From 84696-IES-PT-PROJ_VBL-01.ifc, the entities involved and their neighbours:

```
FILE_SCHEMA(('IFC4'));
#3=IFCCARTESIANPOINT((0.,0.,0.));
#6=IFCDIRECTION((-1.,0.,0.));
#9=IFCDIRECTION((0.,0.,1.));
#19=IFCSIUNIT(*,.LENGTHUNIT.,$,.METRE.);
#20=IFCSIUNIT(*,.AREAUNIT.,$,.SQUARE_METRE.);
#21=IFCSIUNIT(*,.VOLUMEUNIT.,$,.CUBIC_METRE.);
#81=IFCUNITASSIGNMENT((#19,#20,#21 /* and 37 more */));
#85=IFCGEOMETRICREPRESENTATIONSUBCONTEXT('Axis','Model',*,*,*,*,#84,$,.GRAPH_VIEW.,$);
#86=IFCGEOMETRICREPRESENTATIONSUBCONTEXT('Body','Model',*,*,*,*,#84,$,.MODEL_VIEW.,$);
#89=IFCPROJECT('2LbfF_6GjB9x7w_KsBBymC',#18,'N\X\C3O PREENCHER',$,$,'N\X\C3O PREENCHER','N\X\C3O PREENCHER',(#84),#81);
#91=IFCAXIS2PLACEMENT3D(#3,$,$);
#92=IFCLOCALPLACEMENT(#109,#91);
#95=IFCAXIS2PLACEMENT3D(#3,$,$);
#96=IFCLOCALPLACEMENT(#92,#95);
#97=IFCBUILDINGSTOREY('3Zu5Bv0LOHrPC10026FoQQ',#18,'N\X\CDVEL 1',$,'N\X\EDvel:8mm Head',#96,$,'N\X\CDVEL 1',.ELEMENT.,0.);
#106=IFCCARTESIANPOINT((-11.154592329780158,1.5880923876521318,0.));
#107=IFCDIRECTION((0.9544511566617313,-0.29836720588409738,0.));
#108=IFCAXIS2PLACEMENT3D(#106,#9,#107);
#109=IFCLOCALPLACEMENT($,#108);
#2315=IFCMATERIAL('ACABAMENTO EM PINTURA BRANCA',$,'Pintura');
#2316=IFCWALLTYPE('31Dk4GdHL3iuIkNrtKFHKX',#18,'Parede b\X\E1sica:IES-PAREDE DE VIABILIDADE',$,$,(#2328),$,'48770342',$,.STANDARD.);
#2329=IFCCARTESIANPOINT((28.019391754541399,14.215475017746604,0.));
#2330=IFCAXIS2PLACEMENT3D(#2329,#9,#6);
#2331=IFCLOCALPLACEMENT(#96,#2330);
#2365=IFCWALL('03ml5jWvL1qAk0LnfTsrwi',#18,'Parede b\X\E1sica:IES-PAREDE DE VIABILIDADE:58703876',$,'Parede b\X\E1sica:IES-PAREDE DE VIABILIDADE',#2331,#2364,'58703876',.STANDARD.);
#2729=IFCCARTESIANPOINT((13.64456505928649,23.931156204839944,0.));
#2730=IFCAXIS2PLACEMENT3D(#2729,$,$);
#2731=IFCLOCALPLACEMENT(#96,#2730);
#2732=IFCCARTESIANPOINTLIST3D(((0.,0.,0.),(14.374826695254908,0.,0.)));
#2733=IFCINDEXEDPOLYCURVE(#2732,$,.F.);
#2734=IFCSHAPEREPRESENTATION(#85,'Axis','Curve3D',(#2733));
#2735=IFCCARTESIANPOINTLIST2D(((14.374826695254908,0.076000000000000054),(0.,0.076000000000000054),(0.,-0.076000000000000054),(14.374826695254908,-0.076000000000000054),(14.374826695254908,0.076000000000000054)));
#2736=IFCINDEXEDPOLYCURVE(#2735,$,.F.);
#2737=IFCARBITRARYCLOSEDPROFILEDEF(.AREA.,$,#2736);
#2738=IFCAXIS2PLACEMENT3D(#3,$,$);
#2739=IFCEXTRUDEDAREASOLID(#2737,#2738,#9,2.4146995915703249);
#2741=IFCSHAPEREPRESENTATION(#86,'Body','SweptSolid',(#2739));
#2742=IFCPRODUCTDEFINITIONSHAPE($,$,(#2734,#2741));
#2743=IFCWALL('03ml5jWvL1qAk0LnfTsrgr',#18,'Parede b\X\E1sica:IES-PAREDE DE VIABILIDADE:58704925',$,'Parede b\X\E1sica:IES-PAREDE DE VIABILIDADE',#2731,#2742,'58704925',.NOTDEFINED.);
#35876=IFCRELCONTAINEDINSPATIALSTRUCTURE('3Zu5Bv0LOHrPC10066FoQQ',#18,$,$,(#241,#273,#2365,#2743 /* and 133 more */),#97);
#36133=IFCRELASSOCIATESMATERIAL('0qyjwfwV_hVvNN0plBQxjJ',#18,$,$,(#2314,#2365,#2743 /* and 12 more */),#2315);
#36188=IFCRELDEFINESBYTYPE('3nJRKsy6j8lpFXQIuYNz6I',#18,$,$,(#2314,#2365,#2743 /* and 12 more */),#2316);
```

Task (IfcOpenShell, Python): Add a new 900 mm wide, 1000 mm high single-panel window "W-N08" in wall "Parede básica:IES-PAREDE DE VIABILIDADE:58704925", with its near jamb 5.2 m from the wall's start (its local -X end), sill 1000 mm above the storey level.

```python
import numpy as np
import ifcopenshell
import ifcopenshell.api.feature
import ifcopenshell.api.geometry
import ifcopenshell.api.root
import ifcopenshell.api.spatial
import ifcopenshell.geom
import ifcopenshell.util.element
import ifcopenshell.util.placement
import ifcopenshell.util.representation
import ifcopenshell.util.shape
import ifcopenshell.util.unit

model = ifcopenshell.open("84696-IES-PT-PROJ_VBL-01.ifc")
unit_scale = ifcopenshell.util.unit.calculate_unit_scale(model)
settings = ifcopenshell.geom.settings()


def volume(element):
    """Net volume in cubic metres, openings subtracted."""
    shape = ifcopenshell.geom.create_shape(settings, element)
    return ifcopenshell.util.shape.get_volume(shape.geometry)


wall = model.by_id(2743)
storey = ifcopenshell.util.element.get_container(wall, ifc_class="IfcBuildingStorey")
context = ifcopenshell.util.representation.get_context(model, "Model", "Body", "MODEL_VIEW")
before = volume(wall)

width, height, from_end, sill = 0.9, 1, 5.2, 1  # metres

# The wall runs along its own X axis, and the end named is its -X end.
wall_shape = ifcopenshell.geom.create_shape(settings, wall)
x, y, z = ifcopenshell.util.shape.get_vertices(wall_shape.geometry).T
start = x.min() + from_end
face, thickness = float(y.min()), float(y.max() - y.min())
wall_matrix = ifcopenshell.util.placement.get_local_placement(wall.ObjectPlacement)
level = ifcopenshell.util.placement.get_local_placement(storey.ObjectPlacement)[2, 3]


def in_wall(x, y):
    """Placement at x, y metres in the wall's axes, at sill height."""
    matrix = wall_matrix.copy()
    matrix[:, 3] = wall_matrix @ np.array([x / unit_scale, y / unit_scale, 0.0, 1.0])
    matrix[2, 3] = level + sill / unit_scale
    return matrix


# Opening: a box that overshoots both wall faces by 50 mm.
opening = ifcopenshell.api.root.create_entity(model, ifc_class="IfcOpeningElement", predefined_type="OPENING")
box = ifcopenshell.api.geometry.add_wall_representation(
    model, context=context, length=width, height=height, thickness=thickness + 0.1
)
ifcopenshell.api.geometry.assign_representation(model, product=opening, representation=box)
ifcopenshell.api.geometry.edit_object_placement(model, product=opening, matrix=in_wall(start, face - 0.05), is_si=False)
ifcopenshell.api.feature.add_feature(model, feature=opening, element=wall)

window = ifcopenshell.api.root.create_entity(model, ifc_class="IfcWindow", name="W-N08", predefined_type="WINDOW")
window.OverallWidth, window.OverallHeight = width / unit_scale, height / unit_scale
window.PartitioningType = "SINGLE_PANEL"
body = ifcopenshell.api.geometry.add_window_representation(
    model,
    context=context,
    overall_width=window.OverallWidth,
    overall_height=window.OverallHeight,
    partition_type="SINGLE_PANEL",
)
ifcopenshell.api.geometry.assign_representation(model, product=window, representation=body)
ifcopenshell.api.spatial.assign_container(model, products=[window], relating_structure=storey)
ifcopenshell.api.feature.add_filling(model, opening=opening, element=window)

# Centre the window in the wall's thickness.
ifcopenshell.api.geometry.edit_object_placement(model, product=window, matrix=in_wall(start, face), is_si=False)
window_shape = ifcopenshell.geom.create_shape(settings, window)
depth = ifcopenshell.util.shape.get_vertices(window_shape.geometry)[:, 1]
offset = face + thickness / 2 - (depth.min() + depth.max()) / 2
ifcopenshell.api.geometry.edit_object_placement(model, product=window, matrix=in_wall(start, offset), is_si=False)

after = volume(wall)

print(f"wall volume {before:.3f} -> {after:.3f} m3")

model.write("84696-IES-PT-PROJ_VBL-01-out.ifc")
```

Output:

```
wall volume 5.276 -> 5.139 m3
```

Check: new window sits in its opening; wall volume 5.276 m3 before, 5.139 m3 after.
